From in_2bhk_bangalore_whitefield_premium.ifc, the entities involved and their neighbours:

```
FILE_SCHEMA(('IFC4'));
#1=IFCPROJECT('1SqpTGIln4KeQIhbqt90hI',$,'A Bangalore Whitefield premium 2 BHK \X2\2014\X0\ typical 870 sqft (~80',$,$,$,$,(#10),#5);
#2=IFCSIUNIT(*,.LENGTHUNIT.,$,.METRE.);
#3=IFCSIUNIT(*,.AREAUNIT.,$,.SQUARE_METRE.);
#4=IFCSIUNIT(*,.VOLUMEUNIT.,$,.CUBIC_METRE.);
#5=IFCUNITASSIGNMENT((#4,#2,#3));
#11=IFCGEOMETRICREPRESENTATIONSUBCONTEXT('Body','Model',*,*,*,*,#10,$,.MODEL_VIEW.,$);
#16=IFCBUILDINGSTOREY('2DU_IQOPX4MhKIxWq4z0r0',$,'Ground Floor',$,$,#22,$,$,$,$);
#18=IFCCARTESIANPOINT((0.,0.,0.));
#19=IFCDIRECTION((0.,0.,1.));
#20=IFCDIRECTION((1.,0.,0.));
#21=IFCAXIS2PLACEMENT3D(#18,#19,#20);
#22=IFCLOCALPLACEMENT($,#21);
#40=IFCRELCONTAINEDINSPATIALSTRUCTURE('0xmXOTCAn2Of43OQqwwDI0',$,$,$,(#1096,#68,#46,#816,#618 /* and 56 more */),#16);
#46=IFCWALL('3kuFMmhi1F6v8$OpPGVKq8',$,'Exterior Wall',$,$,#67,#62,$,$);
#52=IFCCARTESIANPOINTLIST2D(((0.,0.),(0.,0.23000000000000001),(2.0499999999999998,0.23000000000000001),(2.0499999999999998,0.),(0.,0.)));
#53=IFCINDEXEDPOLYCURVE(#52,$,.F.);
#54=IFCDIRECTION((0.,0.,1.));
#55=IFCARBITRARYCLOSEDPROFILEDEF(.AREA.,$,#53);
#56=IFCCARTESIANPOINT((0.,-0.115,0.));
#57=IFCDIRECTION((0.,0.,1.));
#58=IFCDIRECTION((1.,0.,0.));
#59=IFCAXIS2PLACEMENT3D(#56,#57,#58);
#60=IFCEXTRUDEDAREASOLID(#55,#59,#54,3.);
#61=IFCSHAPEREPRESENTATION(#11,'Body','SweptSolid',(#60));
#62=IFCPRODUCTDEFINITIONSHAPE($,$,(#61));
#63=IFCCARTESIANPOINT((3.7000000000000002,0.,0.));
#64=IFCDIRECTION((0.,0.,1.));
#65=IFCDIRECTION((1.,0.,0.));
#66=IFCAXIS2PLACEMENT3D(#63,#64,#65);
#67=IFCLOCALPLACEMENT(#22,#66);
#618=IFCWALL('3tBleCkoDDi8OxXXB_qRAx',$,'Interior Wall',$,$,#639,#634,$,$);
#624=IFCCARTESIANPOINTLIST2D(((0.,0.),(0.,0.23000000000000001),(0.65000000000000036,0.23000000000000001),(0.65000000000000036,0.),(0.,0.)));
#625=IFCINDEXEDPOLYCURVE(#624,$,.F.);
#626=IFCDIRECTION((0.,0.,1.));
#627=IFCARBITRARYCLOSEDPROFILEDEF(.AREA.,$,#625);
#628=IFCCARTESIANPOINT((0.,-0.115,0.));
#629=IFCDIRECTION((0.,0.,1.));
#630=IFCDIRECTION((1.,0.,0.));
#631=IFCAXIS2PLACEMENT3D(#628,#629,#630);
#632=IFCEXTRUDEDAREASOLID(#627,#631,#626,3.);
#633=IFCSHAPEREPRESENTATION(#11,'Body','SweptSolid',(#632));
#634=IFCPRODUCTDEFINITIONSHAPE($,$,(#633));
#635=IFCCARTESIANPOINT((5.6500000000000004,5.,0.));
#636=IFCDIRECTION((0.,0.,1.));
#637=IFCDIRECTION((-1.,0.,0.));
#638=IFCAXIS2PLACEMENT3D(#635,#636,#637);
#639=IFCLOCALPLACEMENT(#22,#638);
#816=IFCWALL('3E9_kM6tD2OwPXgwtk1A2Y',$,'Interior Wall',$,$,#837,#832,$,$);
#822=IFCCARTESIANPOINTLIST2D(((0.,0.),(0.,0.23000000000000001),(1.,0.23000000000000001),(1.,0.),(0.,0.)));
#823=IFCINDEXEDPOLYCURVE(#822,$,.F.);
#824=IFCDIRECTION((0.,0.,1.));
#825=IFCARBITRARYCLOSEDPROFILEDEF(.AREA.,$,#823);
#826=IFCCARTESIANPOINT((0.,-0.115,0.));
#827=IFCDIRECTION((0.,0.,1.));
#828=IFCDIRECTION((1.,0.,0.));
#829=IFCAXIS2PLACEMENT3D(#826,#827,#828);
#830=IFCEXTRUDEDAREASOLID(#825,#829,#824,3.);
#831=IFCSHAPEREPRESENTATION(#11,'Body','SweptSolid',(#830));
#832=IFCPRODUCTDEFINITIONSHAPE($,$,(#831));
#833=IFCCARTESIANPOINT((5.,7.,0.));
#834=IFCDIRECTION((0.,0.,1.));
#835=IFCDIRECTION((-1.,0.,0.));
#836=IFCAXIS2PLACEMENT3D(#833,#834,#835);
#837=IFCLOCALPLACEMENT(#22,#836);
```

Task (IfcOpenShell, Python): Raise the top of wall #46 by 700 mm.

```python
import ifcopenshell
import ifcopenshell.geom
import ifcopenshell.util.representation
import ifcopenshell.util.shape
import ifcopenshell.util.unit

model = ifcopenshell.open("in_2bhk_bangalore_whitefield_premium.ifc")
unit_scale = ifcopenshell.util.unit.calculate_unit_scale(model)
settings = ifcopenshell.geom.settings()


def volume(element):
    """Net volume in cubic metres, openings subtracted."""
    shape = ifcopenshell.geom.create_shape(settings, element)
    return ifcopenshell.util.shape.get_volume(shape.geometry)


wall = model.by_guid("3kuFMmhi1F6v8$OpPGVKq8")
before = volume(wall)

body = ifcopenshell.util.representation.get_representation(wall, "Model", "Body")
solid = body.Items[0]
old_height = solid.Depth
solid.Depth += 0.7 / unit_scale
after = volume(wall)

print(f"height {old_height:g} -> {solid.Depth:g}, volume {before:.3f} -> {after:.3f} m3")

model.write("in_2bhk_bangalore_whitefield_premium_edited.ifc")
```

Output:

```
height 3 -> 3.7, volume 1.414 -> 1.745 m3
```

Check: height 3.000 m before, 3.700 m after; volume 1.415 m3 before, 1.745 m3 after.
